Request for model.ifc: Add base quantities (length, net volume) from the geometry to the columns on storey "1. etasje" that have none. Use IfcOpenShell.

First a look at what the model holds.

```python
import ifcopenshell
import ifcopenshell.util.element
import ifcopenshell.util.unit

model = ifcopenshell.open("model.ifc")
print(model.schema)
for unit_type in ("LENGTHUNIT", "AREAUNIT", "VOLUMEUNIT"):
    print(unit_type, ifcopenshell.util.unit.calculate_unit_scale(model, unit_type))
storey = next(s for s in model.by_type("IfcBuildingStorey") if s.Name == "1. etasje")
columns = [e for e in ifcopenshell.util.element.get_decomposition(storey) if e.is_a("IfcColumn")]
for e in sorted(columns, key=lambda e: e.id()):
    print(e.id(), e.is_a(), e.Name, list(ifcopenshell.util.element.get_psets(e, qtos_only=True)), sep=" | ")
```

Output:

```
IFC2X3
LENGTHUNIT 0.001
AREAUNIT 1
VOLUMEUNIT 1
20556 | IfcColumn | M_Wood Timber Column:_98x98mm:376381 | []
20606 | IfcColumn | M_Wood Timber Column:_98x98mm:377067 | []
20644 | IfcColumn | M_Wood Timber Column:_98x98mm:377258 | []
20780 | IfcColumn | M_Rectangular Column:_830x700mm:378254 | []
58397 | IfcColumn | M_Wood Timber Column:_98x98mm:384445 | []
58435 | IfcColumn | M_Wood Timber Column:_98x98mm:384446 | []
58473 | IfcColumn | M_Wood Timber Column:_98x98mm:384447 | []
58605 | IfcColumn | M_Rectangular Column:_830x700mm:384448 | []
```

```python
import ifcopenshell
import ifcopenshell.api.pset
import ifcopenshell.geom
import ifcopenshell.util.element
import ifcopenshell.util.shape
import ifcopenshell.util.unit

model = ifcopenshell.open("model.ifc")
unit_scale = ifcopenshell.util.unit.calculate_unit_scale(model)
volume_scale = ifcopenshell.util.unit.calculate_unit_scale(model, "VOLUMEUNIT")
settings = ifcopenshell.geom.settings()

storey = next(s for s in model.by_type("IfcBuildingStorey") if s.Name == "1. etasje")
columns = [e for e in ifcopenshell.util.element.get_decomposition(storey) if e.is_a("IfcColumn")]

for e in sorted(columns, key=lambda e: e.id()):
    if ifcopenshell.util.element.get_psets(e, qtos_only=True, should_inherit=False):
        continue
    # Geometry comes back in metres, in the element's own axes.
    shape = ifcopenshell.geom.create_shape(settings, e)
    values = {
        "Length": ifcopenshell.util.shape.get_z(shape.geometry) / unit_scale,
        "NetVolume": ifcopenshell.util.shape.get_volume(shape.geometry) / volume_scale,
    }
    qto = ifcopenshell.api.pset.add_qto(model, product=e, name="BaseQuantities")
    ifcopenshell.api.pset.edit_qto(model, qto=qto, properties=values)
    print(e.id(), {k: round(v, 3) for k, v in values.items()})

model.write("model_rev.ifc")
```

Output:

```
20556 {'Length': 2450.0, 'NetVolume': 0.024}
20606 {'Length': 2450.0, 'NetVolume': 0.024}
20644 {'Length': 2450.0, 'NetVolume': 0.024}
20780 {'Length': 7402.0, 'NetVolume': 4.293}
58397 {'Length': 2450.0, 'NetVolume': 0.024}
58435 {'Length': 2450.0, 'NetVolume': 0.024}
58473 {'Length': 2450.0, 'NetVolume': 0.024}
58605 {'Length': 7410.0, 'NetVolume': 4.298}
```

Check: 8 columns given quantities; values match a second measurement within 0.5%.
